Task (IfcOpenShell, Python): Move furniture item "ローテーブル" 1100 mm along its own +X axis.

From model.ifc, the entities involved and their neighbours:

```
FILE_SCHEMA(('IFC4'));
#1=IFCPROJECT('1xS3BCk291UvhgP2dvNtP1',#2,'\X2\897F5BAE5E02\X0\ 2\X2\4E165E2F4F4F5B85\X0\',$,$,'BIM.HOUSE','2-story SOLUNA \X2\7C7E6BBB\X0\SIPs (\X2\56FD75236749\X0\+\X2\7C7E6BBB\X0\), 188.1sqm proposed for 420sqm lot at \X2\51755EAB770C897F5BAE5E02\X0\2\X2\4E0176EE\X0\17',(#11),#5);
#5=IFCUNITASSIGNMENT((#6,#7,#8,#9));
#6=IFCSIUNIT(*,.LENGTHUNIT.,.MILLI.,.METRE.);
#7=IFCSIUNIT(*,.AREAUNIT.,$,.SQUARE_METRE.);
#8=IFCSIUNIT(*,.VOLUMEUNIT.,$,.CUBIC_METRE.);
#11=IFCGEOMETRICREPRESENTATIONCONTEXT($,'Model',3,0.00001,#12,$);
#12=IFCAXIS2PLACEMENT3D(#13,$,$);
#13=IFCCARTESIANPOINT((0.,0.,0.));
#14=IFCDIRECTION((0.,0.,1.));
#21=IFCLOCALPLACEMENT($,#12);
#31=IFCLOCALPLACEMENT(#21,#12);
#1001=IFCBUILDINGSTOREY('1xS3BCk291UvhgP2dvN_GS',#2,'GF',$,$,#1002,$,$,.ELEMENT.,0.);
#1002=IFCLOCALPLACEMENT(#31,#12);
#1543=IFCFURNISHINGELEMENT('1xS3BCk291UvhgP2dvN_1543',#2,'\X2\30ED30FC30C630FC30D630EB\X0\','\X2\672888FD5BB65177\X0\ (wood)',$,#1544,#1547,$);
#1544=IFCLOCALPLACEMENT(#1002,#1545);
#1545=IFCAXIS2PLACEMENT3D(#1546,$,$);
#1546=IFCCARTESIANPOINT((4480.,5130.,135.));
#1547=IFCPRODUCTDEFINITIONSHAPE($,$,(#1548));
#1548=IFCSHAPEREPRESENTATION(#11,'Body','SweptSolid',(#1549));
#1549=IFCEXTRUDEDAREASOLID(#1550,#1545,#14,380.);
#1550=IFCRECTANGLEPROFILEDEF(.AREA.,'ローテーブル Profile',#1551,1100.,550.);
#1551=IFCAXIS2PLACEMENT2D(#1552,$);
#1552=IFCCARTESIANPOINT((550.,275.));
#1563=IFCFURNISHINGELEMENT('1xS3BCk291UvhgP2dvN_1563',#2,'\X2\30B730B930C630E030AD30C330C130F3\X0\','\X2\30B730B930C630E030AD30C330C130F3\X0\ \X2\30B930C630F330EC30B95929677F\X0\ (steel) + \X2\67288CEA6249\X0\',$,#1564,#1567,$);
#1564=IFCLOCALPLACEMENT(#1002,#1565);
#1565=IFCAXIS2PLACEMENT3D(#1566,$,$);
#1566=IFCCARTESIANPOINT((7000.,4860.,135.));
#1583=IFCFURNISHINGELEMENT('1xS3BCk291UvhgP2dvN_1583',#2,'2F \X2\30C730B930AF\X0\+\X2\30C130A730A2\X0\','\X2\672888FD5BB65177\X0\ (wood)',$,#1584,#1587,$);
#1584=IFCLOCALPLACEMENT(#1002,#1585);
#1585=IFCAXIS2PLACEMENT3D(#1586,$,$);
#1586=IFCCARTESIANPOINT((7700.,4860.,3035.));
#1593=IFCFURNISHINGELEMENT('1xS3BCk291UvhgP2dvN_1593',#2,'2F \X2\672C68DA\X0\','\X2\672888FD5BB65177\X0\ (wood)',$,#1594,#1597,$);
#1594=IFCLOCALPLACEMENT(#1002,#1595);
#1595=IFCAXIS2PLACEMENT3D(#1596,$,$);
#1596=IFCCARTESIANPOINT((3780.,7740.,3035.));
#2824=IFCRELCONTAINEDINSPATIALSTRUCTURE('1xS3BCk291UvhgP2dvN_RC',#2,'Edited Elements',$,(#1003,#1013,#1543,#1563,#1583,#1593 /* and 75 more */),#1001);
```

```python
import ifcopenshell
import ifcopenshell.api.geometry
import ifcopenshell.util.placement
import ifcopenshell.util.unit

model = ifcopenshell.open("model.ifc")
unit_scale = ifcopenshell.util.unit.calculate_unit_scale(model)

item = model.by_guid("1xS3BCk291UvhgP2dvN_1543")
matrix = ifcopenshell.util.placement.get_local_placement(item.ObjectPlacement)
matrix[:3, 3] += matrix[:3, 0] * 1.1 / unit_scale
ifcopenshell.api.geometry.edit_object_placement(model, product=item, matrix=matrix, is_si=False)

print(ifcopenshell.util.placement.get_local_placement(item.ObjectPlacement).round(3) + 0.0)

model.write("model_rev.ifc")
```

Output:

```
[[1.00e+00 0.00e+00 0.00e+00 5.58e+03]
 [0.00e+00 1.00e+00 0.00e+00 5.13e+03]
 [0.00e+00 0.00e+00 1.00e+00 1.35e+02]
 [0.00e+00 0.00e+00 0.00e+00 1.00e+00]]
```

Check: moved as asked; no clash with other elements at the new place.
